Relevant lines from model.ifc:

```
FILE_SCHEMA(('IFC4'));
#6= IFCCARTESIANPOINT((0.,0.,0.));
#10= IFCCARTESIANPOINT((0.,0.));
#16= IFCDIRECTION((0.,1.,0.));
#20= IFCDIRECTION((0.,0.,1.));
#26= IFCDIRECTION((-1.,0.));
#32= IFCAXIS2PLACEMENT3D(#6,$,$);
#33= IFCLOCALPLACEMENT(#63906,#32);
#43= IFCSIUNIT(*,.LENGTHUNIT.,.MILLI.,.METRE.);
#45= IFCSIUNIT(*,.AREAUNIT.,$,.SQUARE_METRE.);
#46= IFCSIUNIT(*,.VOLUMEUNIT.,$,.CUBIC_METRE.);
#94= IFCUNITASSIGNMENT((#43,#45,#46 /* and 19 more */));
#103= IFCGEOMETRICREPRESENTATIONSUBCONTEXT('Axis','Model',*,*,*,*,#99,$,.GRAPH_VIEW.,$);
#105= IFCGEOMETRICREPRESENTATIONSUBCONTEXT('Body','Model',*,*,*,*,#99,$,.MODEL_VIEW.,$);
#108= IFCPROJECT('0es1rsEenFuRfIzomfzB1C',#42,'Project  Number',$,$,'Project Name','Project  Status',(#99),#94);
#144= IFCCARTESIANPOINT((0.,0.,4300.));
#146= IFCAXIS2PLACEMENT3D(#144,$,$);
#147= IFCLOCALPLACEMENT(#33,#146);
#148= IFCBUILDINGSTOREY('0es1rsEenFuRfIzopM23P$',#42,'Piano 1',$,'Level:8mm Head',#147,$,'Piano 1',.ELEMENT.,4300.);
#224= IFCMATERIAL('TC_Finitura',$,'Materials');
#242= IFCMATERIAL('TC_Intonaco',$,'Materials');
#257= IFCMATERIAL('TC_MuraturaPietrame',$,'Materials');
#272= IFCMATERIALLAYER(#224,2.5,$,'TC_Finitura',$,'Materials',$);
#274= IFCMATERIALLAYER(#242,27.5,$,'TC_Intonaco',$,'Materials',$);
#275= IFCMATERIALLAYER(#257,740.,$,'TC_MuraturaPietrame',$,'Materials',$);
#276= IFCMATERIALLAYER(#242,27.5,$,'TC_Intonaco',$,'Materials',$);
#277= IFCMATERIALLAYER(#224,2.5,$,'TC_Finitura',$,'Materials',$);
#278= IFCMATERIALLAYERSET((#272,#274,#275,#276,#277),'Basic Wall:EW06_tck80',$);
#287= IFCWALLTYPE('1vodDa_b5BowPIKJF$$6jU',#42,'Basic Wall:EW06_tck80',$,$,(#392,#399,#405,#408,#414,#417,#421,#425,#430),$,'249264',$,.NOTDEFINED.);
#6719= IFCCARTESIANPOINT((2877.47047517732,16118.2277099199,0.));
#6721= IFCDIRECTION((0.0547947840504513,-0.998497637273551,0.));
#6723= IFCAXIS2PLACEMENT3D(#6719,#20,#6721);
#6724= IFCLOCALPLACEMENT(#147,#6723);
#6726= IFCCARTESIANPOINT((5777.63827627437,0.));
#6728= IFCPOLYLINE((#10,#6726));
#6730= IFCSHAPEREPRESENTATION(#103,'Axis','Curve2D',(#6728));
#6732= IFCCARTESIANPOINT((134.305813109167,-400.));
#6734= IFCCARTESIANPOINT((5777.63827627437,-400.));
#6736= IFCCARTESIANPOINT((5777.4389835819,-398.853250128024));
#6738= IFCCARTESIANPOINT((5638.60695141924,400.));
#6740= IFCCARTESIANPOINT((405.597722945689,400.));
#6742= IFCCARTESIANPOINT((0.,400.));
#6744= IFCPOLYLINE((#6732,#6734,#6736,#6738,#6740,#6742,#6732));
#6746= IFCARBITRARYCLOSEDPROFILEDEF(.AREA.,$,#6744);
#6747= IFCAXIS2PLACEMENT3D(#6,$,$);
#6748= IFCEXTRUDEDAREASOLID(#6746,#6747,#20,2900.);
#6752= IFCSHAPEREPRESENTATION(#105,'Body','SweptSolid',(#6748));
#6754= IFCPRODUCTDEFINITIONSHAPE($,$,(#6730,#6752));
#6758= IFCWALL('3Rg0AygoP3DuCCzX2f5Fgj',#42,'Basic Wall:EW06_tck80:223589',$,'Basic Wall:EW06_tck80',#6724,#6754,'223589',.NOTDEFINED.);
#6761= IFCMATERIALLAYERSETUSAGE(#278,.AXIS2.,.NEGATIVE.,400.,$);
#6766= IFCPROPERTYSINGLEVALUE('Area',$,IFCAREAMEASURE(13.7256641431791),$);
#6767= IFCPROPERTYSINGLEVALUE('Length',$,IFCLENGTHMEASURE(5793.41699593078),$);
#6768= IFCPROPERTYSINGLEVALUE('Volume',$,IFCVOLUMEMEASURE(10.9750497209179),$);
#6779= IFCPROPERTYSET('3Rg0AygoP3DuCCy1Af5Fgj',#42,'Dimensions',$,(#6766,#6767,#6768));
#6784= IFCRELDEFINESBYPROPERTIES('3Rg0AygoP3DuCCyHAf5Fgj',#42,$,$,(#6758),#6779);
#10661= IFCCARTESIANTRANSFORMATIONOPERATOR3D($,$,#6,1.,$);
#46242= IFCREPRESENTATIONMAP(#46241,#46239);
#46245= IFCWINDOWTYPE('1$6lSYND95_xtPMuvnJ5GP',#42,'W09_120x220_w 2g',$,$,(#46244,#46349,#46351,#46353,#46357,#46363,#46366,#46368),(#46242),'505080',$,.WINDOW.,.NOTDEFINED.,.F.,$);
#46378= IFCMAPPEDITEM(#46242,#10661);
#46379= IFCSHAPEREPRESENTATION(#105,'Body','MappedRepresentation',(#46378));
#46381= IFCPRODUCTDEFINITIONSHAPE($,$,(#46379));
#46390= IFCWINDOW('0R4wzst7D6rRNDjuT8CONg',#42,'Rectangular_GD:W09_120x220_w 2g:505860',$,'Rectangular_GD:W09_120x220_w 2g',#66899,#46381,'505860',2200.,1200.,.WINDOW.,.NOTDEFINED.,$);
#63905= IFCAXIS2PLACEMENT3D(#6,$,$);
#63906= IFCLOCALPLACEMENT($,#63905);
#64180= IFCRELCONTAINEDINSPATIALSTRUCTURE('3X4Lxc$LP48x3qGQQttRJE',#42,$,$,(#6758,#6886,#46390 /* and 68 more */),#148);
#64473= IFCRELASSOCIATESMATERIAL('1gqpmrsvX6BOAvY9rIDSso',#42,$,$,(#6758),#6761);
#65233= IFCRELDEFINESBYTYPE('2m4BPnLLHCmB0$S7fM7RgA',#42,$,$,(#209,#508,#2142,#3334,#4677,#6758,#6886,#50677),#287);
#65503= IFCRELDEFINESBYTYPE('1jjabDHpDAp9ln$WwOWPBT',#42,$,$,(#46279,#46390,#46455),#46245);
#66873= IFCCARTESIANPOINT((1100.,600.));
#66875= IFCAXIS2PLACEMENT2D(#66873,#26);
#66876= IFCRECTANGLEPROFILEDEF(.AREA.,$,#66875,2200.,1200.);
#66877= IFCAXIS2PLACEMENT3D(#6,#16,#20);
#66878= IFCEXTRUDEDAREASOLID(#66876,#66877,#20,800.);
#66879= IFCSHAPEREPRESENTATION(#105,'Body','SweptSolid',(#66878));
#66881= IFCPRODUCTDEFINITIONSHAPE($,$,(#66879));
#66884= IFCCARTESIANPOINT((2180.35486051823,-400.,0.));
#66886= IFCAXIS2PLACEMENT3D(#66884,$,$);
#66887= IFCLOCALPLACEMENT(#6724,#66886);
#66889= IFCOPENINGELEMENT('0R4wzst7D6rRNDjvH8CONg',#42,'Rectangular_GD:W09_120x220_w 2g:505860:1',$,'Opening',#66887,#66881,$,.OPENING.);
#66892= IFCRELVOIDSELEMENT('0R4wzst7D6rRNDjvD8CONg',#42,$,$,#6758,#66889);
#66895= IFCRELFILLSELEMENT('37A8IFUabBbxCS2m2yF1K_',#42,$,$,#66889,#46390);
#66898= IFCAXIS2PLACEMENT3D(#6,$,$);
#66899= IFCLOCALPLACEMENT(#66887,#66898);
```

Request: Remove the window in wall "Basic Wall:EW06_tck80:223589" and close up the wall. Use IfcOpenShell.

```python
import ifcopenshell
import ifcopenshell.api.feature
import ifcopenshell.api.pset
import ifcopenshell.api.root
import ifcopenshell.geom
import ifcopenshell.util.element
import ifcopenshell.util.shape
import ifcopenshell.util.unit

model = ifcopenshell.open("model.ifc")
area_scale = ifcopenshell.util.unit.calculate_unit_scale(model, "AREAUNIT")
volume_scale = ifcopenshell.util.unit.calculate_unit_scale(model, "VOLUMEUNIT")
settings = ifcopenshell.geom.settings()


def volume(element):
    """Net volume in cubic metres, openings subtracted."""
    shape = ifcopenshell.geom.create_shape(settings, element)
    return ifcopenshell.util.shape.get_volume(shape.geometry)


window = model.by_id(46390)
opening = window.FillsVoids[0].RelatingOpeningElement
wall = opening.VoidsElements[0].RelatingBuildingElement
before = volume(wall)

ifcopenshell.api.root.remove_product(model, product=window)
ifcopenshell.api.feature.remove_feature(model, feature=opening)

after = volume(wall)
thickness = 0.8  # wall thickness in metres

# Update the wall's stored quantities.
pset = model.by_id(ifcopenshell.util.element.get_pset(wall, "Dimensions", should_inherit=False)["id"])
ifcopenshell.api.pset.edit_pset(model, pset=pset, properties={
    "Area": model.create_entity("IfcAreaMeasure", after / thickness / area_scale),
    "Volume": model.create_entity("IfcVolumeMeasure", after / volume_scale),
})

print(f"wall volume {before:.3f} -> {after:.3f} m3")

model.write("model_rev.ifc")
```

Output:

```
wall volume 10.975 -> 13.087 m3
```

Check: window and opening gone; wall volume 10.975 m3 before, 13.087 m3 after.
